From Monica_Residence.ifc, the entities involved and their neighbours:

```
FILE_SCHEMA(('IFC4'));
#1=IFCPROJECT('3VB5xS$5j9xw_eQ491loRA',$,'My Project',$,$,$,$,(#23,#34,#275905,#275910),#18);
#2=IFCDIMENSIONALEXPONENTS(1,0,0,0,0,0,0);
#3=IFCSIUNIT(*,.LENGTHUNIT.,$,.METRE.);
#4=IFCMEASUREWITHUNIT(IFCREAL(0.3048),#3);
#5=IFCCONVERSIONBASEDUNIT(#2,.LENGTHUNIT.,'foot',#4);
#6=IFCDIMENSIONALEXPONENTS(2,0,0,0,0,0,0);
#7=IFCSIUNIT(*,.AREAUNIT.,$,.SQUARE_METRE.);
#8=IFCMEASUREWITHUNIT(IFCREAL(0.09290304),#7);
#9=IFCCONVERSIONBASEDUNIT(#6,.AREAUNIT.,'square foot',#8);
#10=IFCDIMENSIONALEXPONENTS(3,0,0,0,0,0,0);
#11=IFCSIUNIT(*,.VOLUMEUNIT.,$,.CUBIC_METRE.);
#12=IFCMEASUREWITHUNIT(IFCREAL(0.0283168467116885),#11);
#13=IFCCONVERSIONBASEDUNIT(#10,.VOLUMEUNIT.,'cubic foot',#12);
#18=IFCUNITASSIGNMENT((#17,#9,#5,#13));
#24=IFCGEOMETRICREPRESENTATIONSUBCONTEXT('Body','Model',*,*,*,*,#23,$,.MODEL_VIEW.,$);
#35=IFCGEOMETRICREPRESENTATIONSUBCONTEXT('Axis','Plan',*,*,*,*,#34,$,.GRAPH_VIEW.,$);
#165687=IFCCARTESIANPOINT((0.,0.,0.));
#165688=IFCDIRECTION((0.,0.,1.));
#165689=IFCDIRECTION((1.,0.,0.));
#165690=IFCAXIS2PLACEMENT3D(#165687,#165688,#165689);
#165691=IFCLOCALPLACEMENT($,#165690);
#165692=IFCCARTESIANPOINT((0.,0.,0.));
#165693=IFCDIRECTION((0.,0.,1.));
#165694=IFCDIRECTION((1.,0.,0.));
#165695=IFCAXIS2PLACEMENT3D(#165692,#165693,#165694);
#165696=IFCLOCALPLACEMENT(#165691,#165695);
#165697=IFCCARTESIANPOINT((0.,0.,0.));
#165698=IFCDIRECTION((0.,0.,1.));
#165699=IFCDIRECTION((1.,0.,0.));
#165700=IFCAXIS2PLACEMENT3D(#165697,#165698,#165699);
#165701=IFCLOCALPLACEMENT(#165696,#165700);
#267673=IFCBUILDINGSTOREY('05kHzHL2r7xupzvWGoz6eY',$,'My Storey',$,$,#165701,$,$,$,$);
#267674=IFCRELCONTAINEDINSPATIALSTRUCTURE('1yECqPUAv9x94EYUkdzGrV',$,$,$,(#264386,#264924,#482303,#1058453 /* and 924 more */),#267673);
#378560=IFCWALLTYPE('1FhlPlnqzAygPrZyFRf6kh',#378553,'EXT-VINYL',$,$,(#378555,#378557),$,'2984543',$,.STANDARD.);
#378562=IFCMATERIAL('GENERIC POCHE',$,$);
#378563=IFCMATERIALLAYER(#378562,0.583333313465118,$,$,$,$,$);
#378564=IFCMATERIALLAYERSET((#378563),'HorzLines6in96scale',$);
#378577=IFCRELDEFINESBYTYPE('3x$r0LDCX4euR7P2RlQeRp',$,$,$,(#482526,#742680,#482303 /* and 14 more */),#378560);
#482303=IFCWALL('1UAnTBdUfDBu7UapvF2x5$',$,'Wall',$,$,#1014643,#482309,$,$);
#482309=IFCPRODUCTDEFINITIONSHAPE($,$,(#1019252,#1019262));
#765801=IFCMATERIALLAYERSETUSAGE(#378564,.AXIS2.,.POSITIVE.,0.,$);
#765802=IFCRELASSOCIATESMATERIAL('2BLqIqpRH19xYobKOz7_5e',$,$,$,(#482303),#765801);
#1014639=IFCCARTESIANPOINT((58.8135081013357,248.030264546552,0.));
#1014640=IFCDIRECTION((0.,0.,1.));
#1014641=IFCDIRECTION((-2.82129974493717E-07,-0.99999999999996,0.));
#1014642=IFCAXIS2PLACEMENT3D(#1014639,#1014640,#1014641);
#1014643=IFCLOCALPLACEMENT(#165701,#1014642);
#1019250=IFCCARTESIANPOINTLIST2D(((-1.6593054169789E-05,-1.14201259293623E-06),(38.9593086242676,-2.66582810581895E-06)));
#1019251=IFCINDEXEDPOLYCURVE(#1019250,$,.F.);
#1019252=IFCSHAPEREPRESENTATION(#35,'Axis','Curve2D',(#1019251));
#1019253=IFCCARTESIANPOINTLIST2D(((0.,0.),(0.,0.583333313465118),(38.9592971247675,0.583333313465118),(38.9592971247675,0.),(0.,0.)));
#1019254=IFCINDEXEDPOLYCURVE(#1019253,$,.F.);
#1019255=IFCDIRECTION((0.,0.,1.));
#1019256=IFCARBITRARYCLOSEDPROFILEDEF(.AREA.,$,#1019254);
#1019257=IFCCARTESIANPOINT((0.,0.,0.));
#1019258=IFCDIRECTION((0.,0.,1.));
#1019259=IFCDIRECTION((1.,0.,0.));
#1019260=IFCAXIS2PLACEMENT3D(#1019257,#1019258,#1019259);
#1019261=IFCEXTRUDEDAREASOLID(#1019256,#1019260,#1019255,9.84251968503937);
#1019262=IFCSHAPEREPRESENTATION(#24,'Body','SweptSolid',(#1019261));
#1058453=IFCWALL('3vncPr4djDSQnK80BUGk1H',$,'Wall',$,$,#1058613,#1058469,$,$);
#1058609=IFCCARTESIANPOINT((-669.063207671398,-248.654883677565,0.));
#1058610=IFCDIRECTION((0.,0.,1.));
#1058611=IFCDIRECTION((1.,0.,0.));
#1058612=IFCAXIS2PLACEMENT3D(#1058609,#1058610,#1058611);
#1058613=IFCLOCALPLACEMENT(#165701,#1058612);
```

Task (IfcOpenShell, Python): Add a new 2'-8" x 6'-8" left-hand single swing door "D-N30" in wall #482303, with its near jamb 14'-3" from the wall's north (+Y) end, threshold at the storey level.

```python
import numpy as np
import ifcopenshell
import ifcopenshell.api.feature
import ifcopenshell.api.geometry
import ifcopenshell.api.root
import ifcopenshell.api.spatial
import ifcopenshell.geom
import ifcopenshell.util.element
import ifcopenshell.util.placement
import ifcopenshell.util.representation
import ifcopenshell.util.shape
import ifcopenshell.util.unit

model = ifcopenshell.open("Monica_Residence.ifc")
unit_scale = ifcopenshell.util.unit.calculate_unit_scale(model)
settings = ifcopenshell.geom.settings()


def volume(element):
    """Net volume in cubic metres, openings subtracted."""
    shape = ifcopenshell.geom.create_shape(settings, element)
    return ifcopenshell.util.shape.get_volume(shape.geometry)


wall = model.by_guid("1UAnTBdUfDBu7UapvF2x5$")
storey = ifcopenshell.util.element.get_container(wall, ifc_class="IfcBuildingStorey")
context = ifcopenshell.util.representation.get_context(model, "Model", "Body", "MODEL_VIEW")
before = volume(wall)

width, height, from_end, sill = 0.8128, 2.032, 4.3434, 0.0  # metres

# The wall runs along its own X axis, and the end named is its -X end.
wall_shape = ifcopenshell.geom.create_shape(settings, wall)
x, y, z = ifcopenshell.util.shape.get_vertices(wall_shape.geometry).T
start = x.min() + from_end
face, thickness = float(y.min()), float(y.max() - y.min())
wall_matrix = ifcopenshell.util.placement.get_local_placement(wall.ObjectPlacement)
level = ifcopenshell.util.placement.get_local_placement(storey.ObjectPlacement)[2, 3]


def in_wall(x, y):
    """Placement at x, y metres in the wall's axes, at sill height."""
    matrix = wall_matrix.copy()
    matrix[:, 3] = wall_matrix @ np.array([x / unit_scale, y / unit_scale, 0.0, 1.0])
    matrix[2, 3] = level + sill / unit_scale
    return matrix


# Opening: a box that overshoots both wall faces by 50 mm.
opening = ifcopenshell.api.root.create_entity(model, ifc_class="IfcOpeningElement", predefined_type="OPENING")
box = ifcopenshell.api.geometry.add_wall_representation(
    model, context=context, length=width, height=height, thickness=thickness + 0.1
)
ifcopenshell.api.geometry.assign_representation(model, product=opening, representation=box)
ifcopenshell.api.geometry.edit_object_placement(model, product=opening, matrix=in_wall(start, face - 0.05), is_si=False)
ifcopenshell.api.feature.add_feature(model, feature=opening, element=wall)

door = ifcopenshell.api.root.create_entity(model, ifc_class="IfcDoor", name="D-N30", predefined_type="DOOR")
door.OverallWidth, door.OverallHeight = width / unit_scale, height / unit_scale
door.OperationType = "SINGLE_SWING_LEFT"
body = ifcopenshell.api.geometry.add_door_representation(
    model,
    context=context,
    overall_width=door.OverallWidth,
    overall_height=door.OverallHeight,
    operation_type="SINGLE_SWING_LEFT",
    lining_properties={"LiningDepth": thickness / unit_scale, "ThresholdDepth": thickness / unit_scale},
)
ifcopenshell.api.geometry.assign_representation(model, product=door, representation=body)
ifcopenshell.api.spatial.assign_container(model, products=[door], relating_structure=storey)
ifcopenshell.api.feature.add_filling(model, opening=opening, element=door)

# The lining spans the wall, so the door starts at the wall face.
ifcopenshell.api.geometry.edit_object_placement(model, product=door, matrix=in_wall(start, face), is_si=False)

after = volume(wall)

print(f"wall volume {before:.3f} -> {after:.3f} m3")

model.write("Monica_Residence_updated.ifc")
```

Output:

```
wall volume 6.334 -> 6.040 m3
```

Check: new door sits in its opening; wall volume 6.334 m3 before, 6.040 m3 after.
